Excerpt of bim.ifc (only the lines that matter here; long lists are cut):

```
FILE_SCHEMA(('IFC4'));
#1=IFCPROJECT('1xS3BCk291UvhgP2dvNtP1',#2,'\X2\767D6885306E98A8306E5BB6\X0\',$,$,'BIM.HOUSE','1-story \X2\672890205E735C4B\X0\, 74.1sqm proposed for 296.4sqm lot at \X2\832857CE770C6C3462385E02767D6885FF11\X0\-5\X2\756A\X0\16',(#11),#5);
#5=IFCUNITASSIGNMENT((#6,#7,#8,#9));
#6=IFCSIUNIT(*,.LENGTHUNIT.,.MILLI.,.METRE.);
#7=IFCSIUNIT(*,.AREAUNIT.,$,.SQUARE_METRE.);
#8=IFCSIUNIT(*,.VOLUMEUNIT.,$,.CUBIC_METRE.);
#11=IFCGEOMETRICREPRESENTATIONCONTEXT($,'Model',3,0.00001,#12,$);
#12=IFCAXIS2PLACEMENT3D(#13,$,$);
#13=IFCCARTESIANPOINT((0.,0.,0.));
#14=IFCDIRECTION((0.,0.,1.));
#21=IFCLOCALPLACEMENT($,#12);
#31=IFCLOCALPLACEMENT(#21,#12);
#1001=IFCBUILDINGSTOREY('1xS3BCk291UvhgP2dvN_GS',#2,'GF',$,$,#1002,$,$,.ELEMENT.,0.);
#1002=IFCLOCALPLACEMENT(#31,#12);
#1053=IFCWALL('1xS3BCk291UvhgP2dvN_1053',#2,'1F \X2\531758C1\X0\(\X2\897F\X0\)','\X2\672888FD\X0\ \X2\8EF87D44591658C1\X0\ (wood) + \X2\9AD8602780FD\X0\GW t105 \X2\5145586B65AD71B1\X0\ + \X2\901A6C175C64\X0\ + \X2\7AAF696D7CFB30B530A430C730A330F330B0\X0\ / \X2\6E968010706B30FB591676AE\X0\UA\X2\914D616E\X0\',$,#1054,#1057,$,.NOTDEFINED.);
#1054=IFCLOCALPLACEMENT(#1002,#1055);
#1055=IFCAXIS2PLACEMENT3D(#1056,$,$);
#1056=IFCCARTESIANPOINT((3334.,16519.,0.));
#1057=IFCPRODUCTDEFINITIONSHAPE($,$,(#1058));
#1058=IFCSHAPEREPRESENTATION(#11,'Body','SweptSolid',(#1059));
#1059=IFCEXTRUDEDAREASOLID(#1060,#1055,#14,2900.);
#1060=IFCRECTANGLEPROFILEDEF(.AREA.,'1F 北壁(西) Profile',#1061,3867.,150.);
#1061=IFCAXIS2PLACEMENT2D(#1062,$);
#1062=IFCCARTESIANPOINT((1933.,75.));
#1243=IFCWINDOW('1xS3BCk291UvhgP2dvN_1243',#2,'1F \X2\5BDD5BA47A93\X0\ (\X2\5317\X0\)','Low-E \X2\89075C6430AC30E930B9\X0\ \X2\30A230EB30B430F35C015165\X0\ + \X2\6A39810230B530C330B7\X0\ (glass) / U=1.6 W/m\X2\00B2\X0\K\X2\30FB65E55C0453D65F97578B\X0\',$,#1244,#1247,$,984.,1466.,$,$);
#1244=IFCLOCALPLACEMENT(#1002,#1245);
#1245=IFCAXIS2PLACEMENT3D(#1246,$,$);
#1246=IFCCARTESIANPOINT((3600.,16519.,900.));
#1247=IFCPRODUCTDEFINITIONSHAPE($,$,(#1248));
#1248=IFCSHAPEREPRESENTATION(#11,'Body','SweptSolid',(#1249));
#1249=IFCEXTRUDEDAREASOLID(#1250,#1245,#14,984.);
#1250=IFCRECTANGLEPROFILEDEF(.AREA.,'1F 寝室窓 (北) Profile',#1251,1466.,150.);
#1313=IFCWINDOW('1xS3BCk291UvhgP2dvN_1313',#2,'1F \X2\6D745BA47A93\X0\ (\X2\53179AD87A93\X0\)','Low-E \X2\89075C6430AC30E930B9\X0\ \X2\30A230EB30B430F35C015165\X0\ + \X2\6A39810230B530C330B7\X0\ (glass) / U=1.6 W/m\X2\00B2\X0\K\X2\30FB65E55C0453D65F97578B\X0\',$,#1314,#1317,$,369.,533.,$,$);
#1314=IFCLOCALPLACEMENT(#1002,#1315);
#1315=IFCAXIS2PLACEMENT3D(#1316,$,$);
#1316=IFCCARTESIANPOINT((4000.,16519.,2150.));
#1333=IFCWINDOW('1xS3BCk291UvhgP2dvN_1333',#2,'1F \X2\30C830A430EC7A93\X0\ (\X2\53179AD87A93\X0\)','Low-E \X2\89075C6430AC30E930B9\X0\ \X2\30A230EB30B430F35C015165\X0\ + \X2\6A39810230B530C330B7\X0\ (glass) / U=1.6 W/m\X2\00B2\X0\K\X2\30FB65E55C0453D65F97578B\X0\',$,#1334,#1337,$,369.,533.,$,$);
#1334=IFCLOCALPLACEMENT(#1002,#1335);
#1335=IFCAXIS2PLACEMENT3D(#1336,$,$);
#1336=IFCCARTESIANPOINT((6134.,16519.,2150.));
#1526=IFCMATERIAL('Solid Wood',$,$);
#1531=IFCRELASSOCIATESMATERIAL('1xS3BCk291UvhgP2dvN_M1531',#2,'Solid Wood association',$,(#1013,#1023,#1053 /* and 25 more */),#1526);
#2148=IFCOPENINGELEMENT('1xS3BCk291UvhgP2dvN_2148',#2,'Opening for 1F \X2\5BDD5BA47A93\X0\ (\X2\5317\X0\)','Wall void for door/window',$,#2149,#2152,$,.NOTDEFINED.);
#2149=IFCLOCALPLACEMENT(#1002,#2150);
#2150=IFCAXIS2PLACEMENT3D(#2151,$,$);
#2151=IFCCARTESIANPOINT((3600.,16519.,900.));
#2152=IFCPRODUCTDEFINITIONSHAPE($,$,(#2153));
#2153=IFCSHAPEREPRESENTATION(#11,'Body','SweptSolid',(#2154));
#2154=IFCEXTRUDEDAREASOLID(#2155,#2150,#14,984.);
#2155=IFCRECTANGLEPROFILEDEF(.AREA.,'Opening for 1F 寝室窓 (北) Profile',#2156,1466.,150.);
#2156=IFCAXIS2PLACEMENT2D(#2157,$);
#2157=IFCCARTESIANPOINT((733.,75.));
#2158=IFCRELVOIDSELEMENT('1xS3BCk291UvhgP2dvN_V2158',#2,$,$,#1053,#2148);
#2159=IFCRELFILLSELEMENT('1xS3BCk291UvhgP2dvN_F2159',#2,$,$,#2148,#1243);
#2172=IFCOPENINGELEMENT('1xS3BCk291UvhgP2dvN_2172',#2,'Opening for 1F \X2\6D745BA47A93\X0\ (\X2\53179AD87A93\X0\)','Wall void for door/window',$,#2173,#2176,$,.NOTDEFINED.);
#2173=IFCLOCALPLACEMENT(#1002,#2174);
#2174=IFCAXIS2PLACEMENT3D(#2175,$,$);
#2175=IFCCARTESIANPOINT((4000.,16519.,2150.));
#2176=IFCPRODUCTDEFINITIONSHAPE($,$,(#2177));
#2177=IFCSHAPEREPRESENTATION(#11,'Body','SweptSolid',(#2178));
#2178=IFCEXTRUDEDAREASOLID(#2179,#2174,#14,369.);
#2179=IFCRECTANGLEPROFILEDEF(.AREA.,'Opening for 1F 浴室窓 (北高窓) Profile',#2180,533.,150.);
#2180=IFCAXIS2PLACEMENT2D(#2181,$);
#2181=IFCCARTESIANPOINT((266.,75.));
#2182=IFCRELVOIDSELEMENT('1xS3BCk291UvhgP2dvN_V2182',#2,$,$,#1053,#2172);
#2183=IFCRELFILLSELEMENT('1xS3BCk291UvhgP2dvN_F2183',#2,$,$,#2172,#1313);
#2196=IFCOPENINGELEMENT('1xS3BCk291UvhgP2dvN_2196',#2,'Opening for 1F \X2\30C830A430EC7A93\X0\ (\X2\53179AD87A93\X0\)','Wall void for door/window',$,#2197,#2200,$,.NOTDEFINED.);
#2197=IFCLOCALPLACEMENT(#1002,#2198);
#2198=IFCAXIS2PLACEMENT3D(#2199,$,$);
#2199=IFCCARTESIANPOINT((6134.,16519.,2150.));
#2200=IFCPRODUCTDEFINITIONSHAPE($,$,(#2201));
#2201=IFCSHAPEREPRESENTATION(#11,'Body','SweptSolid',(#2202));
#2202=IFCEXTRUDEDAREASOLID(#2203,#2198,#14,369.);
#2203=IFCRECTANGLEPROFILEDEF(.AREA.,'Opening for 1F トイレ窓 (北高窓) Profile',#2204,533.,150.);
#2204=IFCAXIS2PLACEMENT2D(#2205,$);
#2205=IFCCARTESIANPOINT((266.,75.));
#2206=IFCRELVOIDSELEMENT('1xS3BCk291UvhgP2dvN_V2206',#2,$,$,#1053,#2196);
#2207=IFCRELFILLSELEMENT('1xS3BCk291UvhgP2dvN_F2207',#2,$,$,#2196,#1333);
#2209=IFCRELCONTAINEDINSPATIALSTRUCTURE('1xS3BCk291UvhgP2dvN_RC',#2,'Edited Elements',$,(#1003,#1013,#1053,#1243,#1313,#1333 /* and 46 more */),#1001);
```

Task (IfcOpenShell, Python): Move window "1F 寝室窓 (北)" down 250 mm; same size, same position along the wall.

```python
import numpy as np
import ifcopenshell
import ifcopenshell.api.geometry
import ifcopenshell.util.placement
import ifcopenshell.util.unit

model = ifcopenshell.open("bim.ifc")
unit_scale = ifcopenshell.util.unit.calculate_unit_scale(model)

window = model.by_guid("1xS3BCk291UvhgP2dvN_1243")
opening = window.FillsVoids[0].RelatingOpeningElement
dz = -0.25 / unit_scale

shift = np.array([0.0, 0.0, dz])
# The window is not placed relative to its opening, so move both.
for product in (opening, window):
    matrix = ifcopenshell.util.placement.get_local_placement(product.ObjectPlacement)
    matrix[:3, 3] += shift
    ifcopenshell.api.geometry.edit_object_placement(model, product=product, matrix=matrix, is_si=False)

print(f"moved by {dz * unit_scale:+.3f} m")

model.write("bim_edited.ifc")
```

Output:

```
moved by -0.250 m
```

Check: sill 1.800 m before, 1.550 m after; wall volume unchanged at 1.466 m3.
